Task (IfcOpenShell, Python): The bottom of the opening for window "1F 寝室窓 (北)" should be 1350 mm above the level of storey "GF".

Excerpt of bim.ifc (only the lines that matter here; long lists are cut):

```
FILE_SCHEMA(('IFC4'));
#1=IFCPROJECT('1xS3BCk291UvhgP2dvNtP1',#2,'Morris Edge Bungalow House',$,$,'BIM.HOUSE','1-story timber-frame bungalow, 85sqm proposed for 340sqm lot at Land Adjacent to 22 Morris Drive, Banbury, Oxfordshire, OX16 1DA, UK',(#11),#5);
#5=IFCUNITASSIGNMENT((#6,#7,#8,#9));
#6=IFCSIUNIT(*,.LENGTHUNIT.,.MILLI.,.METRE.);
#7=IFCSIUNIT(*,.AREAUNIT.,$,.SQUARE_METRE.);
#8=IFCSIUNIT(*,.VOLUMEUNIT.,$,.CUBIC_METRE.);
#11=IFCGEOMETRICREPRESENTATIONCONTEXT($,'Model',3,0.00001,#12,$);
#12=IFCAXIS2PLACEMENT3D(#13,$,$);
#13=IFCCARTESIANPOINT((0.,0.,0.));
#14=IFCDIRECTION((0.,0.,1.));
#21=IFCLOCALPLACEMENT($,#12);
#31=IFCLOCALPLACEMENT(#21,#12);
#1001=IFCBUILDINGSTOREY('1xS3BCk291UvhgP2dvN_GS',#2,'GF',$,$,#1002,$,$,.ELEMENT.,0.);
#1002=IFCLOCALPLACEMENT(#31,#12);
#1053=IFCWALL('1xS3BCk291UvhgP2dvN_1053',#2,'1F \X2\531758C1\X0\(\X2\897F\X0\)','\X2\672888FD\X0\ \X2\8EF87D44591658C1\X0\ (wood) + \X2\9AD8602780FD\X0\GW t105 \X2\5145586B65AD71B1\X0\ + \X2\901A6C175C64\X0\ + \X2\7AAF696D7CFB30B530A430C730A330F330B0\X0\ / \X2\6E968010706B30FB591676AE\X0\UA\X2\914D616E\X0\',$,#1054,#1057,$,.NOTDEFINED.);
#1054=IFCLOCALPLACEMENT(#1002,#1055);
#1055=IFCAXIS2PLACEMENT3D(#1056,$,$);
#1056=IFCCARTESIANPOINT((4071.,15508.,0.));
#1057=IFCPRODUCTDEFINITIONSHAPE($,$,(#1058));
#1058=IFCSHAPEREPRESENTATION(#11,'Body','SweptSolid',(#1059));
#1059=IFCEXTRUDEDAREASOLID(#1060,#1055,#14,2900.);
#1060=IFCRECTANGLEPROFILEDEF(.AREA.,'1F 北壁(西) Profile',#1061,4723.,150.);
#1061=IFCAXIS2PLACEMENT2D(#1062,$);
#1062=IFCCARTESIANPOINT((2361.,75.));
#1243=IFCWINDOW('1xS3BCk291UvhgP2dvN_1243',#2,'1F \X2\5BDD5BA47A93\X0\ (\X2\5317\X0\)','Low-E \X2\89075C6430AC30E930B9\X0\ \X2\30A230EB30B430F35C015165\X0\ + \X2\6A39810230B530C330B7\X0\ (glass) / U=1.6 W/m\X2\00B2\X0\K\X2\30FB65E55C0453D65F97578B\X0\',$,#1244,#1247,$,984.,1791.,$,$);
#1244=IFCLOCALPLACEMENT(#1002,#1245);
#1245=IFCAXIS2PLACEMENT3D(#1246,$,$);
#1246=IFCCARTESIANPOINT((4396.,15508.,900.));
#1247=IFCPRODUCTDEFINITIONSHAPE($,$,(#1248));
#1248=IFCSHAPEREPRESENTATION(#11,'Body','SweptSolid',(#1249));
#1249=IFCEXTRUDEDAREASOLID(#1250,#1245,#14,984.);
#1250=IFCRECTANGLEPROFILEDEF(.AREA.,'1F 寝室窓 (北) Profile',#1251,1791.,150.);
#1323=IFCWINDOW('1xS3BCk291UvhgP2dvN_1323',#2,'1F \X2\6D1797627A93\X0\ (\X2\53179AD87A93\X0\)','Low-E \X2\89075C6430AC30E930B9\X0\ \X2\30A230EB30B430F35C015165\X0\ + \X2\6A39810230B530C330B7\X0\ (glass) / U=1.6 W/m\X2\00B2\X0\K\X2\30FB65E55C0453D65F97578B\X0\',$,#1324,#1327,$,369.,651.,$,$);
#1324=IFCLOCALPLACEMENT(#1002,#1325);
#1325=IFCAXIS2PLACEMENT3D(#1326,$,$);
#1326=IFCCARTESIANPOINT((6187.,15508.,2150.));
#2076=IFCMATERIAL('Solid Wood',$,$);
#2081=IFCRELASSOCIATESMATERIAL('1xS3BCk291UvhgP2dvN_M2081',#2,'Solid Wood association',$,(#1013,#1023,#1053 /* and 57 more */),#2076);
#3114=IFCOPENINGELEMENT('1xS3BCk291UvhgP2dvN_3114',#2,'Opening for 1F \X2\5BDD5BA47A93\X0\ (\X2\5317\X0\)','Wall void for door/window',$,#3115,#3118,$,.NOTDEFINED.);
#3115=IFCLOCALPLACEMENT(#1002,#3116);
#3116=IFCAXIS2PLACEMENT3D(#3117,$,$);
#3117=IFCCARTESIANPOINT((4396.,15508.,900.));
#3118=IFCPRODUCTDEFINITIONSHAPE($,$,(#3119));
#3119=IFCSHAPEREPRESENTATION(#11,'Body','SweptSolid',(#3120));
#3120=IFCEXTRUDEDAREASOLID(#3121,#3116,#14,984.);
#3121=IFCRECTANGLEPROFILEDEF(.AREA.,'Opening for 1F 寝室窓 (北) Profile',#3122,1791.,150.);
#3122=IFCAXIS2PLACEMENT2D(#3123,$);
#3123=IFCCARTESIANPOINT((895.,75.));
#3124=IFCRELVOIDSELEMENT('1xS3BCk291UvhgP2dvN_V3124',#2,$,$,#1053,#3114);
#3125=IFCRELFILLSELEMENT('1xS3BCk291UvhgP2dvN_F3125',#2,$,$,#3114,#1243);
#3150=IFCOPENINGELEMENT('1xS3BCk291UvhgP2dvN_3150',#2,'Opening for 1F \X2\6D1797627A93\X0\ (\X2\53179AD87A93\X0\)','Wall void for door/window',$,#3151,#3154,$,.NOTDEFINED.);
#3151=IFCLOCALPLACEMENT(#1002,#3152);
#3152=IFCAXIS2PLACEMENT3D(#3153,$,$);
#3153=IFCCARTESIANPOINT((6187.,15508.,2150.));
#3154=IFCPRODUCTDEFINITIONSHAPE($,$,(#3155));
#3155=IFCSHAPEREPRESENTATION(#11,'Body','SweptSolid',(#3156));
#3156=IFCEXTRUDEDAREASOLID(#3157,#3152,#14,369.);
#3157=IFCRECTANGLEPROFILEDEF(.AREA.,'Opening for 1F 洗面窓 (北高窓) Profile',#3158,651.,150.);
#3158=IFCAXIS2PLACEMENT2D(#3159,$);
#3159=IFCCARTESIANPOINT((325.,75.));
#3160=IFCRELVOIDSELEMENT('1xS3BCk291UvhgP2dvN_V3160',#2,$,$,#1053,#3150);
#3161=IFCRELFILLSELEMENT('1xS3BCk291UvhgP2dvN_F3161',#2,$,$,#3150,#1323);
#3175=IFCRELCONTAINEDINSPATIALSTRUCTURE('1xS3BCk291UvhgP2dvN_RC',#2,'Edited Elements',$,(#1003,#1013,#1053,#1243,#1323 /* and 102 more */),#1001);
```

```python
import numpy as np
import ifcopenshell
import ifcopenshell.api.geometry
import ifcopenshell.geom
import ifcopenshell.util.element
import ifcopenshell.util.placement
import ifcopenshell.util.shape
import ifcopenshell.util.unit

model = ifcopenshell.open("bim.ifc")
unit_scale = ifcopenshell.util.unit.calculate_unit_scale(model)

window = model.by_guid("1xS3BCk291UvhgP2dvN_1243")
opening = window.FillsVoids[0].RelatingOpeningElement
storey = ifcopenshell.util.element.get_container(window, ifc_class="IfcBuildingStorey")
level = ifcopenshell.util.placement.get_local_placement(storey.ObjectPlacement)[2, 3]

# The opening's origin need not be at the sill, so measure its lowest point.
shape = ifcopenshell.geom.create_shape(ifcopenshell.geom.settings(), opening)
bottom = ifcopenshell.util.shape.get_shape_bottom_elevation(shape, shape.geometry) / unit_scale
dz = level + 1.35 / unit_scale - bottom

shift = np.array([0.0, 0.0, dz])
# The window is not placed relative to its opening, so move both.
for product in (opening, window):
    matrix = ifcopenshell.util.placement.get_local_placement(product.ObjectPlacement)
    matrix[:3, 3] += shift
    ifcopenshell.api.geometry.edit_object_placement(model, product=product, matrix=matrix, is_si=False)

print(f"moved by {dz * unit_scale:+.3f} m")

model.write("bim_edited.ifc")
```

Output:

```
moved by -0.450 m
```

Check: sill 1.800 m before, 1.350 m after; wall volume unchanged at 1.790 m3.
